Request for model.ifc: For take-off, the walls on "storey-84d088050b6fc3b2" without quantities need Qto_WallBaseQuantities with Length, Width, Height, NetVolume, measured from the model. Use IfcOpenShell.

First a look at what the model holds.

```python
import ifcopenshell
import ifcopenshell.util.element
import ifcopenshell.util.unit

model = ifcopenshell.open("model.ifc")
print(model.schema)
for unit_type in ("LENGTHUNIT", "AREAUNIT", "VOLUMEUNIT"):
    print(unit_type, ifcopenshell.util.unit.calculate_unit_scale(model, unit_type))
storey = next(s for s in model.by_type("IfcBuildingStorey") if s.Name == "storey-84d088050b6fc3b2")
walls = [e for e in ifcopenshell.util.element.get_decomposition(storey) if e.is_a("IfcWall")]
for e in sorted(walls, key=lambda e: e.id()):
    print(e.id(), e.is_a(), e.Name, list(ifcopenshell.util.element.get_psets(e, qtos_only=True)), sep=" | ")
```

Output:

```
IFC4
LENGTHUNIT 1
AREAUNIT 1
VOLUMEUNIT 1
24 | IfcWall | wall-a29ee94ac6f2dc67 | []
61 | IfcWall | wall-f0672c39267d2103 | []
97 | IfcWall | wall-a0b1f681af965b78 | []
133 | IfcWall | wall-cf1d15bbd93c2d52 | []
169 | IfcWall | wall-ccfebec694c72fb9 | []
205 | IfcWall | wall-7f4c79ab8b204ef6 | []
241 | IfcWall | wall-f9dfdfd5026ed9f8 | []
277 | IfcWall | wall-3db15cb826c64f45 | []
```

```python
import ifcopenshell
import ifcopenshell.api.pset
import ifcopenshell.geom
import ifcopenshell.util.element
import ifcopenshell.util.shape
import ifcopenshell.util.unit

model = ifcopenshell.open("model.ifc")
unit_scale = ifcopenshell.util.unit.calculate_unit_scale(model)
volume_scale = ifcopenshell.util.unit.calculate_unit_scale(model, "VOLUMEUNIT")
settings = ifcopenshell.geom.settings()

storey = next(s for s in model.by_type("IfcBuildingStorey") if s.Name == "storey-84d088050b6fc3b2")
walls = [e for e in ifcopenshell.util.element.get_decomposition(storey) if e.is_a("IfcWall")]

for e in sorted(walls, key=lambda e: e.id()):
    if ifcopenshell.util.element.get_psets(e, qtos_only=True, should_inherit=False):
        continue
    # Geometry comes back in metres, in the element's own axes.
    shape = ifcopenshell.geom.create_shape(settings, e)
    values = {
        "Length": ifcopenshell.util.shape.get_x(shape.geometry) / unit_scale,
        "Width": ifcopenshell.util.shape.get_y(shape.geometry) / unit_scale,
        "Height": ifcopenshell.util.shape.get_z(shape.geometry) / unit_scale,
        "NetVolume": ifcopenshell.util.shape.get_volume(shape.geometry) / volume_scale,
    }
    qto = ifcopenshell.api.pset.add_qto(model, product=e, name="Qto_WallBaseQuantities")
    ifcopenshell.api.pset.edit_qto(model, qto=qto, properties=values)
    print(e.id(), {k: round(v, 3) for k, v in values.items()})

model.write("model_v2.ifc")
```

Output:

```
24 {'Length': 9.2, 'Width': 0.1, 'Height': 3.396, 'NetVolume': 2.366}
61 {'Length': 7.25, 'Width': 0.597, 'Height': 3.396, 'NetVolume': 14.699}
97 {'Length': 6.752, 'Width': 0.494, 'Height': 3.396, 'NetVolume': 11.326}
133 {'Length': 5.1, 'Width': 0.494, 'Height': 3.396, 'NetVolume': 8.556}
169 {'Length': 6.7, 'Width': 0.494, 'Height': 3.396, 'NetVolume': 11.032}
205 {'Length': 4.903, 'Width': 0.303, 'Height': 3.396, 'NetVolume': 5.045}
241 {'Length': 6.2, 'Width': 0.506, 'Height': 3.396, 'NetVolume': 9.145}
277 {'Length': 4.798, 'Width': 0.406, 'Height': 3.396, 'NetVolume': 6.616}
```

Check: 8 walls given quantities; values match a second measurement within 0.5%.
